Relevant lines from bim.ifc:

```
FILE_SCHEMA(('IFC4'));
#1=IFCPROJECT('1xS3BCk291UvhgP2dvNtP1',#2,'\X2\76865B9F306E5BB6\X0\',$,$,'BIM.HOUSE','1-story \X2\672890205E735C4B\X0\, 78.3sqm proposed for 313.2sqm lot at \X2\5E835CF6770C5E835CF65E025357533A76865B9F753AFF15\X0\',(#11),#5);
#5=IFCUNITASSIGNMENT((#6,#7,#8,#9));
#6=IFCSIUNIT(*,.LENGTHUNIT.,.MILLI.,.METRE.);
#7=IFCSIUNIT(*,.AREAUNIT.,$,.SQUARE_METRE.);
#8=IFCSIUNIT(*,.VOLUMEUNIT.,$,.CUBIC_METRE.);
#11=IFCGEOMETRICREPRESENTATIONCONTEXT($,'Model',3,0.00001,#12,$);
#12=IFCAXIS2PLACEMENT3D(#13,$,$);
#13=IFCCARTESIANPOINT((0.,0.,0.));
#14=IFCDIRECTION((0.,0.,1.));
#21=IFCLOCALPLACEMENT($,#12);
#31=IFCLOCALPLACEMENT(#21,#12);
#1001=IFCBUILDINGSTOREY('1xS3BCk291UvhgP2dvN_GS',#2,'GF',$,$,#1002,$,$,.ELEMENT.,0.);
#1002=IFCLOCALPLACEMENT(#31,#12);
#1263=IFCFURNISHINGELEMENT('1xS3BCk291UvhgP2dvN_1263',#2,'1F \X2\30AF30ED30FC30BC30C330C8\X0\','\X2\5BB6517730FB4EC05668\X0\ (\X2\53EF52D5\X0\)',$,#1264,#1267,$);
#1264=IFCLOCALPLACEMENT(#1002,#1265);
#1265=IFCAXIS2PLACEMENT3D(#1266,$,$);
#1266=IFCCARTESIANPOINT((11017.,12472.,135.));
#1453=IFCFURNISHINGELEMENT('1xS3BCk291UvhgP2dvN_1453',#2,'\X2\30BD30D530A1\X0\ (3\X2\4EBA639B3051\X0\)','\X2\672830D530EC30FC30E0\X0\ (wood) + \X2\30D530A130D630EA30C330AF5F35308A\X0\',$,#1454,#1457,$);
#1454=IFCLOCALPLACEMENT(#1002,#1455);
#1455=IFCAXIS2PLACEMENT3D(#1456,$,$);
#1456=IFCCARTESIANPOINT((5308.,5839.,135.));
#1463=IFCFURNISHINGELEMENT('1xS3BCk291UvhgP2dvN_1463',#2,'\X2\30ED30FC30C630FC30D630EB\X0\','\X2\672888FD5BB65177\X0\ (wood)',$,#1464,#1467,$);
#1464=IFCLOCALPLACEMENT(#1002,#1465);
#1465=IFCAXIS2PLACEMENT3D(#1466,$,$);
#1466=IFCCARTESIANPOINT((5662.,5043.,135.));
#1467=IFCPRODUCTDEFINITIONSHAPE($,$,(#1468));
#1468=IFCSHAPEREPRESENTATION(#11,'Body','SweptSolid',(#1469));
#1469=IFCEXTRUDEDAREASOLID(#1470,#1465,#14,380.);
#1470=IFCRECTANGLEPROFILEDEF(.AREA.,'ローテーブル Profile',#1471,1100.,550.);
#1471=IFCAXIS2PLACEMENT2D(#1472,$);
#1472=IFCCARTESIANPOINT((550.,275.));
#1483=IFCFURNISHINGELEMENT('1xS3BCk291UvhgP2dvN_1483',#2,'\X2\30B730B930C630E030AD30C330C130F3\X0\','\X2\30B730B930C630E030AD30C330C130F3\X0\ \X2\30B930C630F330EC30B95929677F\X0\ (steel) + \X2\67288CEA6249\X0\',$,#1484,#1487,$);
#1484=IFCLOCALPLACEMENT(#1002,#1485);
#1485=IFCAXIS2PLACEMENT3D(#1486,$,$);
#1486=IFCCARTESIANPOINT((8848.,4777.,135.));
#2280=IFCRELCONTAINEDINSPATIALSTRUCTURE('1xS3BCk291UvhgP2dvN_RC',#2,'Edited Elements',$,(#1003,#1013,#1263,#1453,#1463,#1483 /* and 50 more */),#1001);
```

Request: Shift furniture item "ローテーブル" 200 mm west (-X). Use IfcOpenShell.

```python
import ifcopenshell
import ifcopenshell.api.geometry
import ifcopenshell.util.placement

model = ifcopenshell.open("bim.ifc")

item = model.by_guid("1xS3BCk291UvhgP2dvN_1463")
matrix = ifcopenshell.util.placement.get_local_placement(item.ObjectPlacement)
matrix[0, 3] -= 200.0
ifcopenshell.api.geometry.edit_object_placement(model, product=item, matrix=matrix, is_si=False)

print(ifcopenshell.util.placement.get_local_placement(item.ObjectPlacement).round(3) + 0.0)

model.write("bim_rev.ifc")
```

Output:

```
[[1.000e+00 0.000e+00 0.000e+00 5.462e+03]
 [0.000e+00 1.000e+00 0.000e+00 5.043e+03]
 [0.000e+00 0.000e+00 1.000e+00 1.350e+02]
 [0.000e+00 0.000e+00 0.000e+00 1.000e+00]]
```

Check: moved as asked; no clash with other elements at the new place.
